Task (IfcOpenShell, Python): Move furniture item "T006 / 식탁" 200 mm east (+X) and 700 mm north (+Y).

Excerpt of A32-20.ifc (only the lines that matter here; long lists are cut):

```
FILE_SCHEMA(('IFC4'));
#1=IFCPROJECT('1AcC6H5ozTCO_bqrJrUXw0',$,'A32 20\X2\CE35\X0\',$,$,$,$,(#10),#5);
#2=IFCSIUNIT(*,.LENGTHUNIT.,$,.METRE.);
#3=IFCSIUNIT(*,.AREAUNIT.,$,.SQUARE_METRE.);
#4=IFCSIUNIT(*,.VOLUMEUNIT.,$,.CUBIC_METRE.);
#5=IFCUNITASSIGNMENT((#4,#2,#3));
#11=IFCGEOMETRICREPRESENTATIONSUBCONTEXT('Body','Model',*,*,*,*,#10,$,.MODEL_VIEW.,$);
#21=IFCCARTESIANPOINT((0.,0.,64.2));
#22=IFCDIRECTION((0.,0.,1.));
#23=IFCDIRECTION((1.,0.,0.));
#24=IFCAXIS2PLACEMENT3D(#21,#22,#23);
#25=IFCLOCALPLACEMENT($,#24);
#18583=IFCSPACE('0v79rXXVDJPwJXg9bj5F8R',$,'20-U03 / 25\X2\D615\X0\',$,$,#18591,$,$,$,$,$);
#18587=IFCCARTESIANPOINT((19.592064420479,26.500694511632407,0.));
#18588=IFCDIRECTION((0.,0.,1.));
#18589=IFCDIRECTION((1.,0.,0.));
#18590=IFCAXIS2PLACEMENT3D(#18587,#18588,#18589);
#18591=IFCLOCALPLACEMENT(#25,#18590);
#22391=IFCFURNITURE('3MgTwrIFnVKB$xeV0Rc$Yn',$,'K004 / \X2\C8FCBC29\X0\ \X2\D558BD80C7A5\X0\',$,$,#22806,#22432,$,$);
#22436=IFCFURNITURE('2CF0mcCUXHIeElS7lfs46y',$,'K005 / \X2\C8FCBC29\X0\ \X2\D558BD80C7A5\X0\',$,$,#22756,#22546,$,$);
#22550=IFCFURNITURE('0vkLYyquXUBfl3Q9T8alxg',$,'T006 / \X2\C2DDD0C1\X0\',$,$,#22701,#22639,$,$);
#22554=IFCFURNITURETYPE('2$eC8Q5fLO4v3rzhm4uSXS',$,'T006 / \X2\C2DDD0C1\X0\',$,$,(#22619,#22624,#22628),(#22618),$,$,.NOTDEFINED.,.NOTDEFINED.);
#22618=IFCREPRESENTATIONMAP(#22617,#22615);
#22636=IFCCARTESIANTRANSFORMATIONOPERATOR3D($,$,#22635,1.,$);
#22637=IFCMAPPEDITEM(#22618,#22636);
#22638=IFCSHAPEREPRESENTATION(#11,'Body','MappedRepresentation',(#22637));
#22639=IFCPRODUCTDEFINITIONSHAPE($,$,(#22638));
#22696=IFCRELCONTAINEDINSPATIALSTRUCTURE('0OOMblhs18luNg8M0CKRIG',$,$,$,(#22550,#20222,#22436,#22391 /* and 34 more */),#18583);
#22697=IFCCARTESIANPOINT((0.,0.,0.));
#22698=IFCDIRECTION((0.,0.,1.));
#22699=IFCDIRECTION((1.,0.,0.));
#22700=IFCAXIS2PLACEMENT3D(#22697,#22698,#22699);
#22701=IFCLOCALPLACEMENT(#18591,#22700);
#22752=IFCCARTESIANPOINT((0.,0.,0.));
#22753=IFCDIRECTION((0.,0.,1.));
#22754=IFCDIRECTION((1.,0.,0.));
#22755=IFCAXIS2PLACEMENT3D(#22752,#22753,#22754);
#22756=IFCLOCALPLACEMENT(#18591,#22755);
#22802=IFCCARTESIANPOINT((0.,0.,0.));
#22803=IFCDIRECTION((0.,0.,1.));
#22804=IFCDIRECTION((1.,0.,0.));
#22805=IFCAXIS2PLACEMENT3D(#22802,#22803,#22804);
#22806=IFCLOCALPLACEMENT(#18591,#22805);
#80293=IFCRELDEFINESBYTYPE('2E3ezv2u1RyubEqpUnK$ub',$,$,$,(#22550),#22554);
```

```python
import ifcopenshell
import ifcopenshell.api.geometry
import ifcopenshell.util.placement
import ifcopenshell.util.unit

model = ifcopenshell.open("A32-20.ifc")
unit_scale = ifcopenshell.util.unit.calculate_unit_scale(model)

item = model.by_guid("0vkLYyquXUBfl3Q9T8alxg")
matrix = ifcopenshell.util.placement.get_local_placement(item.ObjectPlacement)
matrix[0, 3] += 0.2 / unit_scale
matrix[1, 3] += 0.7 / unit_scale
ifcopenshell.api.geometry.edit_object_placement(model, product=item, matrix=matrix, is_si=False)

print(ifcopenshell.util.placement.get_local_placement(item.ObjectPlacement).round(3) + 0.0)

model.write("A32-20_v2.ifc")
```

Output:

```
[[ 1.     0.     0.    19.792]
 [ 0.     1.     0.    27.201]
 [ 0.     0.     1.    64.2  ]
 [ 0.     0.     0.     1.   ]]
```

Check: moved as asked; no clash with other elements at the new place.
